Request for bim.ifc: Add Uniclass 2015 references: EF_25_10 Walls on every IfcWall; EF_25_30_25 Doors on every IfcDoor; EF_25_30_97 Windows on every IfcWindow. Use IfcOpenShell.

First a look at what the model holds.

```python
import ifcopenshell

model = ifcopenshell.open("bim.ifc")
print(model.schema)
print("classifications:", [c.Name for c in model.by_type("IfcClassification")])
for ifc_class in ("IfcDoor", "IfcRoof", "IfcStair", "IfcWall", "IfcWindow"):
    print(ifc_class, len(model.by_type(ifc_class)))
```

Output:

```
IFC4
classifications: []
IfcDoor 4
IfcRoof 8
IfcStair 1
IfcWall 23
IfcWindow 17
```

```python
import ifcopenshell
import ifcopenshell.api.classification

model = ifcopenshell.open("bim.ifc")

system = ifcopenshell.api.classification.add_classification(model, classification="Uniclass 2015")

codes = {
    "IfcWall": ("EF_25_10", "Walls"),
    "IfcDoor": ("EF_25_30_25", "Doors"),
    "IfcWindow": ("EF_25_30_97", "Windows"),
}
for ifc_class, (code, name) in codes.items():
    products = model.by_type(ifc_class)
    ifcopenshell.api.classification.add_reference(
        model, products=products, classification=system, identification=code, name=name
    )
    print(code, len(products))

model.write("bim_updated.ifc")
```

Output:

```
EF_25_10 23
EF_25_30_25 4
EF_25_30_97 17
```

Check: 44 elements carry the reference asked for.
